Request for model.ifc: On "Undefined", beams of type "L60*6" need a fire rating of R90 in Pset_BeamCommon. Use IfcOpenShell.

First a look at what the model holds.

```python
import ifcopenshell
import ifcopenshell.util.element

model = ifcopenshell.open("model.ifc")
print(model.schema)
storey = next(s for s in model.by_type("IfcBuildingStorey") if s.Name == "Undefined")
beams = [e for e in ifcopenshell.util.element.get_decomposition(storey) if e.is_a("IfcBeam")]
seen = {}
for e in beams:
    element_type = ifcopenshell.util.element.get_type(e)
    key = (element_type.Name if element_type != e and element_type else None, ifcopenshell.util.element.get_pset(e, "Pset_BeamCommon", "FireRating"))
    seen[key] = seen.get(key, 0) + 1
for (name, value), count in sorted(seen.items(), key=str):
    print(count, "x", name, "|", value)
```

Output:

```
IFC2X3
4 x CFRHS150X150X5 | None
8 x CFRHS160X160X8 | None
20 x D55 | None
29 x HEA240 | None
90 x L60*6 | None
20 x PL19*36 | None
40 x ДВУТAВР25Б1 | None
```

```python
import ifcopenshell
import ifcopenshell.api.pset
import ifcopenshell.util.element

model = ifcopenshell.open("model.ifc")

storey = next(s for s in model.by_type("IfcBuildingStorey") if s.Name == "Undefined")
beams = [e for e in ifcopenshell.util.element.get_decomposition(storey) if e.is_a("IfcBeam")]

count = 0
for e in beams:
    element_type = ifcopenshell.util.element.get_type(e)
    if element_type in (None, e) or element_type.Name != "L60*6":
        continue
    # add_pset returns the element's existing set when there is one.
    pset = ifcopenshell.api.pset.add_pset(model, product=e, name="Pset_BeamCommon")
    ifcopenshell.api.pset.edit_pset(model, pset=pset, properties={"FireRating": "R90"})
    count += 1

print(count, "beams updated")

model.write("model_updated.ifc")
```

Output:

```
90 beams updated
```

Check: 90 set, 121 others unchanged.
